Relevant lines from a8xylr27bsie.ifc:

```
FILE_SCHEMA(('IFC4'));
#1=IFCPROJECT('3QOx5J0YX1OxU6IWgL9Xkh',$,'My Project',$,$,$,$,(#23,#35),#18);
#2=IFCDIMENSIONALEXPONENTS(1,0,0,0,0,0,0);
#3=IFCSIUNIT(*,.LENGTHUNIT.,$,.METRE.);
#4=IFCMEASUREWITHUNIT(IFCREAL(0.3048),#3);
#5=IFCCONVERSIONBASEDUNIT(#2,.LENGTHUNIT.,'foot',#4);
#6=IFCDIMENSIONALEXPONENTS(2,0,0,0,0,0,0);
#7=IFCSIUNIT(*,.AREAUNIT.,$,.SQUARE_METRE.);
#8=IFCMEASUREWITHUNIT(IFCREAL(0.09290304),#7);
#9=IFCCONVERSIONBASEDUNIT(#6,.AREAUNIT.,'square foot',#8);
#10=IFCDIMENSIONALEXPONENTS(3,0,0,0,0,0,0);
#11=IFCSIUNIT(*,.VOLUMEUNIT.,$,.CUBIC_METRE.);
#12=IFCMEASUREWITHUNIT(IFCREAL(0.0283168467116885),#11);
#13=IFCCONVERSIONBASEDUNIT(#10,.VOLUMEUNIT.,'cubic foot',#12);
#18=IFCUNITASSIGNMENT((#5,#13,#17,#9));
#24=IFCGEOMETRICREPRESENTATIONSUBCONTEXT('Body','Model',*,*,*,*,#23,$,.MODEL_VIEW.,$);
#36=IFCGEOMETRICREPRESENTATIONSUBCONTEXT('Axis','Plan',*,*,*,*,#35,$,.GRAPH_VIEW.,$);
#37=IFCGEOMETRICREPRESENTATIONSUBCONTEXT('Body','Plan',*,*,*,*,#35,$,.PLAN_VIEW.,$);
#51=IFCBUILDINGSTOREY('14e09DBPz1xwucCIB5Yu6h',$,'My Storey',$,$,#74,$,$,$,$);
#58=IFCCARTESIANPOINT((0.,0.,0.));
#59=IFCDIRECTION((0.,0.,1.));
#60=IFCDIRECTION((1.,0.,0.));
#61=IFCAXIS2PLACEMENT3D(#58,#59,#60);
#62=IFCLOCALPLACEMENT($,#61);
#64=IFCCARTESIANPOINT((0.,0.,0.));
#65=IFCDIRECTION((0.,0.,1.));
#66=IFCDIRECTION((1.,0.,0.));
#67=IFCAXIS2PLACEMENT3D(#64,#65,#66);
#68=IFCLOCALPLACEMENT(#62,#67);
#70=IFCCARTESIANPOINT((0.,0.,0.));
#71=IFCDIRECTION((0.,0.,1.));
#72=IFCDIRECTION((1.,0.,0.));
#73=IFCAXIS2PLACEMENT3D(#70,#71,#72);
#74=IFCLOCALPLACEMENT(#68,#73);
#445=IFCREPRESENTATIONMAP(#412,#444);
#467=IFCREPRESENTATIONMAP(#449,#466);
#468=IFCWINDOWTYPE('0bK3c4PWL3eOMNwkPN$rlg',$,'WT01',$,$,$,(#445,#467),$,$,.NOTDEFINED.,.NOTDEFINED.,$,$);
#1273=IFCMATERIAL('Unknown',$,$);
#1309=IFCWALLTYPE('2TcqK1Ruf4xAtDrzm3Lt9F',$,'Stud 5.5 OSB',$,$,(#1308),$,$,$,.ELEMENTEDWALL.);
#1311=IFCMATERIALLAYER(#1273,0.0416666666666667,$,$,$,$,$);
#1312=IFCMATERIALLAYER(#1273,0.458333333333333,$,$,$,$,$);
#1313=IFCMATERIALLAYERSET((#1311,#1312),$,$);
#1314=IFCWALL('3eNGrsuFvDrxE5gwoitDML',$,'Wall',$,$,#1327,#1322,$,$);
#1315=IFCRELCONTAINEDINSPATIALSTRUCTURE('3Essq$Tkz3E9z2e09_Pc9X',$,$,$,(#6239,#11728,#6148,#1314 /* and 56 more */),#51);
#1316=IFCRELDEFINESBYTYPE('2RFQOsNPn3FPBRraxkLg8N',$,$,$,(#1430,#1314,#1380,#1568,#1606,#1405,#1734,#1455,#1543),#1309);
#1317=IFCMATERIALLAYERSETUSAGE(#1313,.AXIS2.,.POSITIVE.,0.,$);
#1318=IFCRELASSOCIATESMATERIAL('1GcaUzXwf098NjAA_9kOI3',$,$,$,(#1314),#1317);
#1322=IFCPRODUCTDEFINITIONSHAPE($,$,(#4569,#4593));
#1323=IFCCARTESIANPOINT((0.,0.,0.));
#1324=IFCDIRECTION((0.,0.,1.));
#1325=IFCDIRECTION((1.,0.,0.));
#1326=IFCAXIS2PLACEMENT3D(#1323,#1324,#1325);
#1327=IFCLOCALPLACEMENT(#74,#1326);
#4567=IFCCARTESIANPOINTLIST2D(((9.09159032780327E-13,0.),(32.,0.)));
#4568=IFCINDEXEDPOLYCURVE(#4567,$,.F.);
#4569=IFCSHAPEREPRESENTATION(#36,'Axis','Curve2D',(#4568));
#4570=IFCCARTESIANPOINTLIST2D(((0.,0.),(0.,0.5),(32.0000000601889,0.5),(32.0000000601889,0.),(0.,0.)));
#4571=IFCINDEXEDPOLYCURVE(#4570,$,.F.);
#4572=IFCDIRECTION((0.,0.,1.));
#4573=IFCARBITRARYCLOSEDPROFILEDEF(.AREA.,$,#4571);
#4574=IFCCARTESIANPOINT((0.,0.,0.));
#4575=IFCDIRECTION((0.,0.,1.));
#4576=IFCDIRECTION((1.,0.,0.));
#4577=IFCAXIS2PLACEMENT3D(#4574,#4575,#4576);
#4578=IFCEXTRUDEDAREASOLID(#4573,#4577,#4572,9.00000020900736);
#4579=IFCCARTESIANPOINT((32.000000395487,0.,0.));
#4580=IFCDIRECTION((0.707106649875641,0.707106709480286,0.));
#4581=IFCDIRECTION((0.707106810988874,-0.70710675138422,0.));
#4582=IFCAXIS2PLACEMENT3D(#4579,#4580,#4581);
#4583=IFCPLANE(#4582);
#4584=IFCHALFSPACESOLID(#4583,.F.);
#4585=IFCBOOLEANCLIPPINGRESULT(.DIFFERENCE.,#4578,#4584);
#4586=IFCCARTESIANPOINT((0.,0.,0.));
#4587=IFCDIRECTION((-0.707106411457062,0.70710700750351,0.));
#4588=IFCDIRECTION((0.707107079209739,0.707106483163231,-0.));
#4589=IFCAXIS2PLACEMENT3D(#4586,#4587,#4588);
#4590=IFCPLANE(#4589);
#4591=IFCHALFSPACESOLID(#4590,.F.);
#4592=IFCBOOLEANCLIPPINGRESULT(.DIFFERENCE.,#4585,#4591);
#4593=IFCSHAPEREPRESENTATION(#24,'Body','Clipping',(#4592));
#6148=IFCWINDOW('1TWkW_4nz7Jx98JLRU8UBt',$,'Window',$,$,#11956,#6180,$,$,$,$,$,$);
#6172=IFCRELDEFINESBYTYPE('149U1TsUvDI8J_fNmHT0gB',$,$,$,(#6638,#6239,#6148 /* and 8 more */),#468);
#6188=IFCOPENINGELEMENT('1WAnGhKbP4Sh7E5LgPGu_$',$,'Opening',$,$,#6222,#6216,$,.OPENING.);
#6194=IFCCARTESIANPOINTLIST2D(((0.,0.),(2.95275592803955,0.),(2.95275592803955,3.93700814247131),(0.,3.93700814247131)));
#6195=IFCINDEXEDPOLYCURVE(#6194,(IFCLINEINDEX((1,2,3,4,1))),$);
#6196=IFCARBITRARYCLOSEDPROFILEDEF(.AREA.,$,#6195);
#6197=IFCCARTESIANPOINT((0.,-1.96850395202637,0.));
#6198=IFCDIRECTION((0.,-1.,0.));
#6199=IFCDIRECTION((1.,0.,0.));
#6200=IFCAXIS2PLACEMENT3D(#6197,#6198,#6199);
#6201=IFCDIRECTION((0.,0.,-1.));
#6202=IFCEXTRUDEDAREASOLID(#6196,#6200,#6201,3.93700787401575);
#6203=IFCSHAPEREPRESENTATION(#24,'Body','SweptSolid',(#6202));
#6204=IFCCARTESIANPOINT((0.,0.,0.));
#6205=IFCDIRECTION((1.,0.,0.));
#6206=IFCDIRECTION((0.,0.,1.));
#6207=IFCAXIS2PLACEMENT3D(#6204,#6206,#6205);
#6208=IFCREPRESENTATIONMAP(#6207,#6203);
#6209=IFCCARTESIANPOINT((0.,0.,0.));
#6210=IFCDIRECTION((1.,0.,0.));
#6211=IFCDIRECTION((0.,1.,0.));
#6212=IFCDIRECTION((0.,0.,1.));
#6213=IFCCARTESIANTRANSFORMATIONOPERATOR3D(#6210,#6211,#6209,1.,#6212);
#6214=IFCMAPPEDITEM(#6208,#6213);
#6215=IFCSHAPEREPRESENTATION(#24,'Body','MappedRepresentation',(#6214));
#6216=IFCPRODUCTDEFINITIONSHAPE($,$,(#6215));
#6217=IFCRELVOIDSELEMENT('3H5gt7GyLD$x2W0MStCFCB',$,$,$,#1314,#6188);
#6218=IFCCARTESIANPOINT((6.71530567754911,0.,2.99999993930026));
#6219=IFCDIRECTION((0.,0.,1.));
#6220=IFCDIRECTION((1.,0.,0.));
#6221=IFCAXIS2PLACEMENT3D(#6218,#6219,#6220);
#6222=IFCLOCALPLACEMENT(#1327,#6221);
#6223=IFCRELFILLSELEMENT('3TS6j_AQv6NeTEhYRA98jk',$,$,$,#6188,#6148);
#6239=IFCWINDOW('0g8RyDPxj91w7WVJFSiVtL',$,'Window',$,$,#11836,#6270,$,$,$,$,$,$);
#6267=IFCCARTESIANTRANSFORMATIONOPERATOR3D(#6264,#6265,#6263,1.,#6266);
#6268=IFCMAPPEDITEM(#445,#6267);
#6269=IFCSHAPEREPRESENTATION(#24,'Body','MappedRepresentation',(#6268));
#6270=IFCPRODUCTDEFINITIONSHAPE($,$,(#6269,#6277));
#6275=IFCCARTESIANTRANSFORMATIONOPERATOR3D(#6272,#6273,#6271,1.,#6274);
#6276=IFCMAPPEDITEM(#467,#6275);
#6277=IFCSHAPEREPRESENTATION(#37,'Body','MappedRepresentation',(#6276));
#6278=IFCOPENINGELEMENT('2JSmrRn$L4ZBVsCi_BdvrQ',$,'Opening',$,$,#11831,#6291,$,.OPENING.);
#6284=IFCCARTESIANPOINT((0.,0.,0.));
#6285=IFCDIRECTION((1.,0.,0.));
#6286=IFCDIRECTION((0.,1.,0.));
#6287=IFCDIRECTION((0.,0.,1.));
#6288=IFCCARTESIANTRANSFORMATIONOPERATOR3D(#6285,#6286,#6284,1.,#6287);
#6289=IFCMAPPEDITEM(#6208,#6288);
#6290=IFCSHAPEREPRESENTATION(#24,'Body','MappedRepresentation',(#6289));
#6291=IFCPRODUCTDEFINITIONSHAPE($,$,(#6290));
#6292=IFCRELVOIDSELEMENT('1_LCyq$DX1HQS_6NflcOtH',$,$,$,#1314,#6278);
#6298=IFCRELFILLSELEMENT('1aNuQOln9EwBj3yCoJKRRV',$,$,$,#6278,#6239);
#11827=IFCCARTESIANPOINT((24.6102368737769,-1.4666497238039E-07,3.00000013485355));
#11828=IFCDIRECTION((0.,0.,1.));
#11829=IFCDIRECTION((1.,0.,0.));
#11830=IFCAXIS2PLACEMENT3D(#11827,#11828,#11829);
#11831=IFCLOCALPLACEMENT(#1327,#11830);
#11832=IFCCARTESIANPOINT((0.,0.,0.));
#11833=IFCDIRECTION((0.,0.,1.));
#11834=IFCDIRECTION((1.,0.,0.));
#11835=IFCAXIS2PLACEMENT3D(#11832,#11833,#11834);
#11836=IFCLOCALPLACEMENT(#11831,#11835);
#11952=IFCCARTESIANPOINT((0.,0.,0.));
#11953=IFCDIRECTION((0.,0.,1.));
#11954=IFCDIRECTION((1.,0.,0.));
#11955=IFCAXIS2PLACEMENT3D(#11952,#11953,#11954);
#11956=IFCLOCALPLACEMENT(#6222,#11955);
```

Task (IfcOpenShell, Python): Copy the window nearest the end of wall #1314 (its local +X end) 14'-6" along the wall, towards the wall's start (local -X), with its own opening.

```python
import ifcopenshell
import ifcopenshell.api.feature
import ifcopenshell.api.geometry
import ifcopenshell.api.root
import ifcopenshell.geom
import ifcopenshell.util.element
import ifcopenshell.util.placement
import ifcopenshell.util.shape
import ifcopenshell.util.unit

model = ifcopenshell.open("a8xylr27bsie.ifc")
unit_scale = ifcopenshell.util.unit.calculate_unit_scale(model)
settings = ifcopenshell.geom.settings()


def volume(element):
    """Net volume in cubic metres, openings subtracted."""
    shape = ifcopenshell.geom.create_shape(settings, element)
    return ifcopenshell.util.shape.get_volume(shape.geometry)


window = model.by_guid("0g8RyDPxj91w7WVJFSiVtL")
opening = window.FillsVoids[0].RelatingOpeningElement
wall = opening.VoidsElements[0].RelatingBuildingElement
before = volume(wall)
shift = ifcopenshell.util.placement.get_local_placement(wall.ObjectPlacement)[:3, 0] * -174 * 0.0254 / unit_scale

# copy_class copies the void relationship, type, container and properties, but no geometry.
new_opening = ifcopenshell.api.root.copy_class(model, product=opening)
new_opening.Representation = ifcopenshell.util.element.copy_deep(
    model, opening.Representation, exclude=["IfcGeometricRepresentationContext", "IfcRepresentationMap"]
)
new_window = ifcopenshell.api.root.copy_class(model, product=window)
new_window.Representation = ifcopenshell.util.element.copy_deep(
    model, window.Representation, exclude=["IfcGeometricRepresentationContext", "IfcRepresentationMap"]
)
ifcopenshell.api.feature.add_filling(model, opening=new_opening, element=new_window)

for old, new in ((opening, new_opening), (window, new_window)):
    matrix = ifcopenshell.util.placement.get_local_placement(old.ObjectPlacement)
    matrix[:3, 3] += shift
    ifcopenshell.api.geometry.edit_object_placement(model, product=new, matrix=matrix, is_si=False)

after = volume(wall)

print(f"wall volume {before:.3f} -> {after:.3f} m3")

model.write("a8xylr27bsie_v2.ifc")
```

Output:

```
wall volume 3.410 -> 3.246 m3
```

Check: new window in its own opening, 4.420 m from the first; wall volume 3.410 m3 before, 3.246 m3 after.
